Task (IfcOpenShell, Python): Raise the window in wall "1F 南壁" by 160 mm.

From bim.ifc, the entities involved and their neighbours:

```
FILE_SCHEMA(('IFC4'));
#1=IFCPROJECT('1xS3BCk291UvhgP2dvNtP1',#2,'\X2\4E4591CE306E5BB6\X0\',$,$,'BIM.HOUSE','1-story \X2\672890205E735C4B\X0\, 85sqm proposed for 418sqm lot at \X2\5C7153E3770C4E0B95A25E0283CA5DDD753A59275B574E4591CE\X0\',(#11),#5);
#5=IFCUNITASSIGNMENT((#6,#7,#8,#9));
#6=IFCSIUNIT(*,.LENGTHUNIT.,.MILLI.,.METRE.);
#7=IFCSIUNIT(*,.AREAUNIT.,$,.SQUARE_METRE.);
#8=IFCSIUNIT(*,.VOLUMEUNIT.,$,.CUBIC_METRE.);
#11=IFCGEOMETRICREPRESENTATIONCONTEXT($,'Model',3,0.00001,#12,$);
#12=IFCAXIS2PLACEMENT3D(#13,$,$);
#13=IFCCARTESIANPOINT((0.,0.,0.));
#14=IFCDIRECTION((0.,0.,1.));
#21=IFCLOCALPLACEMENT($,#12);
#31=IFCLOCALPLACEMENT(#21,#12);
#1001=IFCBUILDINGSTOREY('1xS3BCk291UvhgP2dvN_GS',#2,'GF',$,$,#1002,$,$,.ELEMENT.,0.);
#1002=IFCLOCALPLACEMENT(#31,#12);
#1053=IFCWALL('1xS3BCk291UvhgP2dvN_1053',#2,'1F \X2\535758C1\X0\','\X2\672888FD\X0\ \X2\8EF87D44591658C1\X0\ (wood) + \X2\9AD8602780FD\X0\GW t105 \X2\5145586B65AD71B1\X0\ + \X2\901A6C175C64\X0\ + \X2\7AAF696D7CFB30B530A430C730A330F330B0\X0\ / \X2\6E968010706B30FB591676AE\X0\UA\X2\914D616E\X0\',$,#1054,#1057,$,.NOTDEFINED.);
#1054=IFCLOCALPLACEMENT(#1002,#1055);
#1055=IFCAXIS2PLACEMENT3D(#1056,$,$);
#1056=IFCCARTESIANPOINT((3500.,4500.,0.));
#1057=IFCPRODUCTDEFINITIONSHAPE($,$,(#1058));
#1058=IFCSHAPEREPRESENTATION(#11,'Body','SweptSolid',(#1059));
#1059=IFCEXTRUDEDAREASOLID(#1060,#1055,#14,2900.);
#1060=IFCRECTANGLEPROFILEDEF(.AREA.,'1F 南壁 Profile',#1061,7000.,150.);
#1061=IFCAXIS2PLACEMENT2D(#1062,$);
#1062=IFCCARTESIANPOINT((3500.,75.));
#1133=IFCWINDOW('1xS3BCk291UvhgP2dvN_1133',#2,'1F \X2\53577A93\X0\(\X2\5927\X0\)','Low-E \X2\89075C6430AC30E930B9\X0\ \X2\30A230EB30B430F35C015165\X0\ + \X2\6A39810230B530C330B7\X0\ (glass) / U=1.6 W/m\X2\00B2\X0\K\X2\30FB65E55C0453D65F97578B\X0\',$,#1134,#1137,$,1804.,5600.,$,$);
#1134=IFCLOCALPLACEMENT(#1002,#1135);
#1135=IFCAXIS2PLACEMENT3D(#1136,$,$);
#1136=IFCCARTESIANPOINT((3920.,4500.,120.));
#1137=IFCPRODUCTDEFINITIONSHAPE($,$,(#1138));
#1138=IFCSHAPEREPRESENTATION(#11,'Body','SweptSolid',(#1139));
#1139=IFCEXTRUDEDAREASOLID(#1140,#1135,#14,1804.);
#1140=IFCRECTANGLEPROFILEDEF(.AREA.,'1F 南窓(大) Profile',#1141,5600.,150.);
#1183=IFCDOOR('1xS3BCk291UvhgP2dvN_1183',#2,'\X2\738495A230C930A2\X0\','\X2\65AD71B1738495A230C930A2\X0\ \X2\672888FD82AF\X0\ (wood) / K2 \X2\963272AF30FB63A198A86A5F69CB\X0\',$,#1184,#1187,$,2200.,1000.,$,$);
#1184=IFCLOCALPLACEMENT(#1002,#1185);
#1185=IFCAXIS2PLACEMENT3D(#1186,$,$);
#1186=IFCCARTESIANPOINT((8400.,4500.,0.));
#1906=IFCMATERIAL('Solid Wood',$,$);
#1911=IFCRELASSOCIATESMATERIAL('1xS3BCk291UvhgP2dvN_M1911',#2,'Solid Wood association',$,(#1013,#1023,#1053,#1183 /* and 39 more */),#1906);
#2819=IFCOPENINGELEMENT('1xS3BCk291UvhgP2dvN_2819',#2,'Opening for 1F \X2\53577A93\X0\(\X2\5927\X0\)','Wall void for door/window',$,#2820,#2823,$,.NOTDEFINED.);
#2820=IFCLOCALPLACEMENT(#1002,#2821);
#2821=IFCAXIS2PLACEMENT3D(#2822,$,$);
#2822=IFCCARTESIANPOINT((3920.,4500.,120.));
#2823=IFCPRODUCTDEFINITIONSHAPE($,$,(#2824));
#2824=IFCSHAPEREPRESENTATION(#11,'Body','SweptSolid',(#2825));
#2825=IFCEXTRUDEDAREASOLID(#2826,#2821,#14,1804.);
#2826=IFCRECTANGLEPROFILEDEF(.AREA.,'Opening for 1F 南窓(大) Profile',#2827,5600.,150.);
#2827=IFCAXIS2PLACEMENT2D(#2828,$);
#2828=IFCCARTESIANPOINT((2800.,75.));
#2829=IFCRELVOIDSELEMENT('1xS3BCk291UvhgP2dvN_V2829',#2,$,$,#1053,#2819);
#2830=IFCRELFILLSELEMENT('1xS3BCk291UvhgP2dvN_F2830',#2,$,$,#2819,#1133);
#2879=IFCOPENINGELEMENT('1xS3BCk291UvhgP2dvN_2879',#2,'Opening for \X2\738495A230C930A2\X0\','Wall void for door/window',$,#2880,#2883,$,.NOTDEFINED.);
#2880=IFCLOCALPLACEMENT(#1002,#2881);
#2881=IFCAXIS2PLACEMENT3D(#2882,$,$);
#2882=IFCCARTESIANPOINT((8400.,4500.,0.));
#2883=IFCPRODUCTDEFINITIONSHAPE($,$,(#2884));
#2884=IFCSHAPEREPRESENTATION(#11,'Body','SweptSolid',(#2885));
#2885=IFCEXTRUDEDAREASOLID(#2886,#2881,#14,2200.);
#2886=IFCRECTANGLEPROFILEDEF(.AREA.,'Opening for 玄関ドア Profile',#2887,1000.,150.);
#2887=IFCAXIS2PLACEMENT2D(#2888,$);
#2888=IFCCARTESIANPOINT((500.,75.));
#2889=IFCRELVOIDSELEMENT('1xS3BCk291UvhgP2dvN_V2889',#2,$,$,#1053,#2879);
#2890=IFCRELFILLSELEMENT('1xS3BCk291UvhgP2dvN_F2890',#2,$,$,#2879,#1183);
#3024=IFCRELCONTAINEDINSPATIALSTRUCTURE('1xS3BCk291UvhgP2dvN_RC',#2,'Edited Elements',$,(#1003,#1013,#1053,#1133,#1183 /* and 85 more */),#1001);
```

```python
import numpy as np
import ifcopenshell
import ifcopenshell.api.geometry
import ifcopenshell.util.placement
import ifcopenshell.util.unit

model = ifcopenshell.open("bim.ifc")
unit_scale = ifcopenshell.util.unit.calculate_unit_scale(model)

window = model.by_guid("1xS3BCk291UvhgP2dvN_1133")
opening = window.FillsVoids[0].RelatingOpeningElement
dz = 160.0

shift = np.array([0.0, 0.0, dz])
# The window is not placed relative to its opening, so move both.
for product in (opening, window):
    matrix = ifcopenshell.util.placement.get_local_placement(product.ObjectPlacement)
    matrix[:3, 3] += shift
    ifcopenshell.api.geometry.edit_object_placement(model, product=product, matrix=matrix, is_si=False)

print(f"moved by {dz * unit_scale:+.3f} m")

model.write("bim_rev.ifc")
```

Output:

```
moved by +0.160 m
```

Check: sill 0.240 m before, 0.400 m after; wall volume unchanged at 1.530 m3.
